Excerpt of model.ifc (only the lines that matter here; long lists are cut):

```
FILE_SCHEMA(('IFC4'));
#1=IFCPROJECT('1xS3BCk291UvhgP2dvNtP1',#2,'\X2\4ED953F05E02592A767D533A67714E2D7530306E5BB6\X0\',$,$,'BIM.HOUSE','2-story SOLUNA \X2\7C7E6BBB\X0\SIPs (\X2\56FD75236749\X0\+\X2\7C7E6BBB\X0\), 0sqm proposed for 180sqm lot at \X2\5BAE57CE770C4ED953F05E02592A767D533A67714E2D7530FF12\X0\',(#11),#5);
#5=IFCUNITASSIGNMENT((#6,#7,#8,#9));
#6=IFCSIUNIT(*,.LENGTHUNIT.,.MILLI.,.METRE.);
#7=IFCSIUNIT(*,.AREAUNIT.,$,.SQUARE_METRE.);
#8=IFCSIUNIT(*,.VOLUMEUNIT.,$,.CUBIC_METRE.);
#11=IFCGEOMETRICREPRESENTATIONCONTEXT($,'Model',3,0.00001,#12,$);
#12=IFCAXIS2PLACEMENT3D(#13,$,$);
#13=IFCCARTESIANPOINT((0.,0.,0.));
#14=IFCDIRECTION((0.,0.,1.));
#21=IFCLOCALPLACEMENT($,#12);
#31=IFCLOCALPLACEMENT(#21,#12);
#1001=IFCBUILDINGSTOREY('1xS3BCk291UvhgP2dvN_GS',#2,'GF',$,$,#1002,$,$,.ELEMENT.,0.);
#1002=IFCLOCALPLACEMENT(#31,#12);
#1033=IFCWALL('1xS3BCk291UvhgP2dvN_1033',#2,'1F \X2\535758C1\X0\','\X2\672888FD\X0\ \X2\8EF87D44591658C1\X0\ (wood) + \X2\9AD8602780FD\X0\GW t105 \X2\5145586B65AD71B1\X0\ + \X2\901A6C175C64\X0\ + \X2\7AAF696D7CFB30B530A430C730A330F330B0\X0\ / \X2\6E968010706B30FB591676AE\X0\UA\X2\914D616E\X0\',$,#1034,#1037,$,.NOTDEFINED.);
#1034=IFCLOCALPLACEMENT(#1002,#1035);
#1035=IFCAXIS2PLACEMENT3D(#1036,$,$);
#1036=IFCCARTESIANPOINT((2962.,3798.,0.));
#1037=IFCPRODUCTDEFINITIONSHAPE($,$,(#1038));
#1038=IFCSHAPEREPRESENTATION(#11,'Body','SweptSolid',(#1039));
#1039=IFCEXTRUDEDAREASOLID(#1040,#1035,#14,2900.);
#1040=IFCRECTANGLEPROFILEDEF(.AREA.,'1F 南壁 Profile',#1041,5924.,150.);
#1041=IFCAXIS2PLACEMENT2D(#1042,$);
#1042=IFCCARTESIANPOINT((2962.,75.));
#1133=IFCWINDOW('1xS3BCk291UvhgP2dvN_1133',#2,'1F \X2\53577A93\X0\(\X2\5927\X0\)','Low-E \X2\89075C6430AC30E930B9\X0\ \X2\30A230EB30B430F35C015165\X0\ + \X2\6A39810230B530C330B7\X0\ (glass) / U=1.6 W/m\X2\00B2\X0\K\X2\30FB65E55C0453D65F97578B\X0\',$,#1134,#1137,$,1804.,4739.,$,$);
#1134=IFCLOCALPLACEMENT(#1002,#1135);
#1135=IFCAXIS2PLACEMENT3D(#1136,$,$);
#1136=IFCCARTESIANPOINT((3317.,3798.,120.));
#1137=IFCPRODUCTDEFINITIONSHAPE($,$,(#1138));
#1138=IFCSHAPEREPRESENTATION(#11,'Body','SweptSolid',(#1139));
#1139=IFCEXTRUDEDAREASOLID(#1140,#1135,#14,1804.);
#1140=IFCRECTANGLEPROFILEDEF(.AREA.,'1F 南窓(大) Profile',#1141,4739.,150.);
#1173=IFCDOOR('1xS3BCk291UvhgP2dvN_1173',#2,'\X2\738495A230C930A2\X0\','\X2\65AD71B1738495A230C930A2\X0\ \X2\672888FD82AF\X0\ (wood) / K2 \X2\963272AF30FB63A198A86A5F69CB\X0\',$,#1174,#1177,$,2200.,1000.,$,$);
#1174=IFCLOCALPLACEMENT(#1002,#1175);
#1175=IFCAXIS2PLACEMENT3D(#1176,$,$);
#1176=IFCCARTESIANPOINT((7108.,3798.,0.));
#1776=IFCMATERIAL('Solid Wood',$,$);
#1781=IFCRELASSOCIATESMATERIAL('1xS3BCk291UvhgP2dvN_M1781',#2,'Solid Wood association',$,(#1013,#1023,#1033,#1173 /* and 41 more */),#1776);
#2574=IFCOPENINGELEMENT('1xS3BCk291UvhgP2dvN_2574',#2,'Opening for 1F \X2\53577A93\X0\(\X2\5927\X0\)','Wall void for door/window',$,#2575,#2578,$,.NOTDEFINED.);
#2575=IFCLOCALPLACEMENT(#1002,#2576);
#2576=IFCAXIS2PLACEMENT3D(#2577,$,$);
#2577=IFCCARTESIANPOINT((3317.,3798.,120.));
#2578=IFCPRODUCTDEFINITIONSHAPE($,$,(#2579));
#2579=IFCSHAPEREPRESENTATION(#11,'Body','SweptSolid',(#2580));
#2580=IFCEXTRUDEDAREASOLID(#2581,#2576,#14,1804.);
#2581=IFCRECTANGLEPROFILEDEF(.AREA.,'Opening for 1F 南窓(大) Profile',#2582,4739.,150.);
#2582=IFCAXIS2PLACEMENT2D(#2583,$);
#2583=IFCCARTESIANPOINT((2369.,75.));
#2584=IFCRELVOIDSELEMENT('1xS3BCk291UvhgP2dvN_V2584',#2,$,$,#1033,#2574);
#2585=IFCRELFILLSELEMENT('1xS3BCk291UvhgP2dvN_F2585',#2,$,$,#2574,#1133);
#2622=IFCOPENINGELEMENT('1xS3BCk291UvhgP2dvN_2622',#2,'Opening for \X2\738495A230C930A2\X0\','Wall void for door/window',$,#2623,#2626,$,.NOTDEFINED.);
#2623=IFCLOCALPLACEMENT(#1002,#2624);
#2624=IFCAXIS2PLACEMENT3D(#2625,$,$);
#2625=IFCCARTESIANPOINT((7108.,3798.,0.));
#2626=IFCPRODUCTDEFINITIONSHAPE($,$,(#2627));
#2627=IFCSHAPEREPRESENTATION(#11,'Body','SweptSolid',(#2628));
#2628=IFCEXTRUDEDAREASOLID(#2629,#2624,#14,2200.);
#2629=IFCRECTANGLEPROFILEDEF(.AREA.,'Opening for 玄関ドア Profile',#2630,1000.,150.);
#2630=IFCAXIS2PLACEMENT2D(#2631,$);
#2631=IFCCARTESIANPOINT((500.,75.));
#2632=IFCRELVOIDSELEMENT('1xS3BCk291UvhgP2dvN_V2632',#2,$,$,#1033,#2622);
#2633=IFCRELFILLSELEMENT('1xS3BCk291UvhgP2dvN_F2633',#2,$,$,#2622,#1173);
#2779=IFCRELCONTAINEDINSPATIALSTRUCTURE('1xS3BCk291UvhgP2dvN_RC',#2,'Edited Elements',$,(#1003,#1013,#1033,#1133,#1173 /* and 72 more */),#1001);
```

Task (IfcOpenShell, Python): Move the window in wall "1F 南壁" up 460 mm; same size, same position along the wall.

```python
import numpy as np
import ifcopenshell
import ifcopenshell.api.geometry
import ifcopenshell.util.placement
import ifcopenshell.util.unit

model = ifcopenshell.open("model.ifc")
unit_scale = ifcopenshell.util.unit.calculate_unit_scale(model)

window = model.by_guid("1xS3BCk291UvhgP2dvN_1133")
opening = window.FillsVoids[0].RelatingOpeningElement
dz = 0.46 / unit_scale

shift = np.array([0.0, 0.0, dz])
# The window is not placed relative to its opening, so move both.
for product in (opening, window):
    matrix = ifcopenshell.util.placement.get_local_placement(product.ObjectPlacement)
    matrix[:3, 3] += shift
    ifcopenshell.api.geometry.edit_object_placement(model, product=product, matrix=matrix, is_si=False)

print(f"moved by {dz * unit_scale:+.3f} m")

model.write("model_rev.ifc")
```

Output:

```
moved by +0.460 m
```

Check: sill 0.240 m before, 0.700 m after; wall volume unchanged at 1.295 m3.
